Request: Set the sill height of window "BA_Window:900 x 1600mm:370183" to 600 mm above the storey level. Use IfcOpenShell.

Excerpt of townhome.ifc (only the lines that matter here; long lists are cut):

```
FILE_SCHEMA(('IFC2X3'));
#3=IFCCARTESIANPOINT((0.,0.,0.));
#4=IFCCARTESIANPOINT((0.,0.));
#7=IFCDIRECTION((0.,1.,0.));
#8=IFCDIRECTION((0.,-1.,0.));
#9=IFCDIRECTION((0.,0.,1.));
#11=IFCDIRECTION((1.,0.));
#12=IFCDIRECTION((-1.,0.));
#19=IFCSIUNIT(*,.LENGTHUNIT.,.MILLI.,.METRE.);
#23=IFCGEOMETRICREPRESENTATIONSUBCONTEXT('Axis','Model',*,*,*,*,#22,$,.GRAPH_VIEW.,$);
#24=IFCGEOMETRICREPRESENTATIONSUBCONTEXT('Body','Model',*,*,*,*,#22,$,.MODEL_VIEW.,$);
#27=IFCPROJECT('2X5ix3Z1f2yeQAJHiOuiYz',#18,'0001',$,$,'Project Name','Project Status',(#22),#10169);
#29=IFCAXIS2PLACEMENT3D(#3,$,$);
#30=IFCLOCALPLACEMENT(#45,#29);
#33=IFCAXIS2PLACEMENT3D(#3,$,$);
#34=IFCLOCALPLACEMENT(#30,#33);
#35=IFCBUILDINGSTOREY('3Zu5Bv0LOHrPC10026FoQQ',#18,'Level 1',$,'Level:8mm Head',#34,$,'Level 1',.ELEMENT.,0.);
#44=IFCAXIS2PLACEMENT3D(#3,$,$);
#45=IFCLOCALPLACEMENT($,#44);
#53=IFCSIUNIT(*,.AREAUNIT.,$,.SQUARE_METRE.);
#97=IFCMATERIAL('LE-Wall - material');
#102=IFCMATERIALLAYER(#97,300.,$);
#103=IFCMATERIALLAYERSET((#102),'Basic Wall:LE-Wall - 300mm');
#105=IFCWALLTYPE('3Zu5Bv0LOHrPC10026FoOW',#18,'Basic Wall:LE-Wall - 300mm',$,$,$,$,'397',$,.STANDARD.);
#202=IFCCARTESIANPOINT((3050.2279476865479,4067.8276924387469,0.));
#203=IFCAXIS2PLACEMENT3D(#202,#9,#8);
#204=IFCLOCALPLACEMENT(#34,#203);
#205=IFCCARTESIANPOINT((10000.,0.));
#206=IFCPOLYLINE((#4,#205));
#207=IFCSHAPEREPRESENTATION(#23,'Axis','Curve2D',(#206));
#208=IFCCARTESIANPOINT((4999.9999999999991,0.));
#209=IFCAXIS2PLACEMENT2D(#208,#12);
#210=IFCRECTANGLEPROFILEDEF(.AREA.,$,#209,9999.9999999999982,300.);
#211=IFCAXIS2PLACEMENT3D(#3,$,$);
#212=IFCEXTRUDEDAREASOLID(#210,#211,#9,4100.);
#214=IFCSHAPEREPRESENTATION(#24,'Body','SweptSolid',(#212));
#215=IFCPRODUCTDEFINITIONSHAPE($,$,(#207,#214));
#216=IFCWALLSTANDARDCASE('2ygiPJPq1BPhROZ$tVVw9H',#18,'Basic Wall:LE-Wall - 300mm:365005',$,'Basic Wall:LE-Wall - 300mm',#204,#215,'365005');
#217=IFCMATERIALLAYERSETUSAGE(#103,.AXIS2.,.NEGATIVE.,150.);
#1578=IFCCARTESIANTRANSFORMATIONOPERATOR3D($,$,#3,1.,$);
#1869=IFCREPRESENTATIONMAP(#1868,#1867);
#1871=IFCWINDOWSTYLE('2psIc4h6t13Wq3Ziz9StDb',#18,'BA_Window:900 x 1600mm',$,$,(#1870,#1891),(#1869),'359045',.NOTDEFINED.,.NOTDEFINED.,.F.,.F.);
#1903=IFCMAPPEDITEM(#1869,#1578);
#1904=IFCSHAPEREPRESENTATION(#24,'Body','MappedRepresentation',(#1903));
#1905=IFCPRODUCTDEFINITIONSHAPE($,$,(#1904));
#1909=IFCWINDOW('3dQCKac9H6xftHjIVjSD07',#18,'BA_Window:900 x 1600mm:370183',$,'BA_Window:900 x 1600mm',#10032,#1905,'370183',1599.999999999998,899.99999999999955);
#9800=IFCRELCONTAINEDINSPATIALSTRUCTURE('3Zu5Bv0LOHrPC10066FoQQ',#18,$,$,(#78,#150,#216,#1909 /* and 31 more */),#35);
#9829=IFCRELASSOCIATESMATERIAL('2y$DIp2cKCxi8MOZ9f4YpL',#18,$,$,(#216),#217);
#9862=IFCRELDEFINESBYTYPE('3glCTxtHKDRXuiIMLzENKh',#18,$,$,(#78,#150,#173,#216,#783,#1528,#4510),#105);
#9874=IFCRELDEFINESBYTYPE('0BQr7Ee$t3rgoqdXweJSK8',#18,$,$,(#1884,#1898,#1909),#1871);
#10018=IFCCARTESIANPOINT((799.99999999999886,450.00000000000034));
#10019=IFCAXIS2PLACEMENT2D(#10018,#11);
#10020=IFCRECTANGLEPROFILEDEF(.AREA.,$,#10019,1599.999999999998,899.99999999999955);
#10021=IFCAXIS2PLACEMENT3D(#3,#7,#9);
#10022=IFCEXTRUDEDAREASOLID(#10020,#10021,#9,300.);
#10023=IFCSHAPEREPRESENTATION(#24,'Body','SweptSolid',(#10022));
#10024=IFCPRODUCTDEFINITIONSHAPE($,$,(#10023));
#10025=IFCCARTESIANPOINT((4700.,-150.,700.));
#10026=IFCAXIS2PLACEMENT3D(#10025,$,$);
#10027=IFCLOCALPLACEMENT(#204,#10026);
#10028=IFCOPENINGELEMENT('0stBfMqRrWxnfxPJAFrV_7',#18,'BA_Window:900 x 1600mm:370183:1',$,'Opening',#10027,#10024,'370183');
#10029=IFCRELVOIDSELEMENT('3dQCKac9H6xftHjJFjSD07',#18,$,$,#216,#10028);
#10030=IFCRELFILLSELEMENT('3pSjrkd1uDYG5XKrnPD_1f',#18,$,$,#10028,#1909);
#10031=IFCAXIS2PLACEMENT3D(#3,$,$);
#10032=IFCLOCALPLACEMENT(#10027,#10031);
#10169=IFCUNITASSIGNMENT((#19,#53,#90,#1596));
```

```python
import numpy as np
import ifcopenshell
import ifcopenshell.api.geometry
import ifcopenshell.geom
import ifcopenshell.util.element
import ifcopenshell.util.placement
import ifcopenshell.util.shape
import ifcopenshell.util.unit

model = ifcopenshell.open("townhome.ifc")
unit_scale = ifcopenshell.util.unit.calculate_unit_scale(model)

window = model.by_guid("3dQCKac9H6xftHjIVjSD07")
opening = window.FillsVoids[0].RelatingOpeningElement
storey = ifcopenshell.util.element.get_container(window, ifc_class="IfcBuildingStorey")
level = ifcopenshell.util.placement.get_local_placement(storey.ObjectPlacement)[2, 3]

# The opening's origin need not be at the sill, so measure its lowest point.
shape = ifcopenshell.geom.create_shape(ifcopenshell.geom.settings(), opening)
bottom = ifcopenshell.util.shape.get_shape_bottom_elevation(shape, shape.geometry) / unit_scale
dz = level + 600.0 - bottom

shift = np.array([0.0, 0.0, dz])
# The window is placed relative to its opening, so it follows when the opening moves.
matrix = ifcopenshell.util.placement.get_local_placement(opening.ObjectPlacement)
matrix[:3, 3] += shift
ifcopenshell.api.geometry.edit_object_placement(
    model, product=opening, matrix=matrix, is_si=False, should_transform_children=True
)

print(f"moved by {dz * unit_scale:+.3f} m")

model.write("townhome_edited.ifc")
```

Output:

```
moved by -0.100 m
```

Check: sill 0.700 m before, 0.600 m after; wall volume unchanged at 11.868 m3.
